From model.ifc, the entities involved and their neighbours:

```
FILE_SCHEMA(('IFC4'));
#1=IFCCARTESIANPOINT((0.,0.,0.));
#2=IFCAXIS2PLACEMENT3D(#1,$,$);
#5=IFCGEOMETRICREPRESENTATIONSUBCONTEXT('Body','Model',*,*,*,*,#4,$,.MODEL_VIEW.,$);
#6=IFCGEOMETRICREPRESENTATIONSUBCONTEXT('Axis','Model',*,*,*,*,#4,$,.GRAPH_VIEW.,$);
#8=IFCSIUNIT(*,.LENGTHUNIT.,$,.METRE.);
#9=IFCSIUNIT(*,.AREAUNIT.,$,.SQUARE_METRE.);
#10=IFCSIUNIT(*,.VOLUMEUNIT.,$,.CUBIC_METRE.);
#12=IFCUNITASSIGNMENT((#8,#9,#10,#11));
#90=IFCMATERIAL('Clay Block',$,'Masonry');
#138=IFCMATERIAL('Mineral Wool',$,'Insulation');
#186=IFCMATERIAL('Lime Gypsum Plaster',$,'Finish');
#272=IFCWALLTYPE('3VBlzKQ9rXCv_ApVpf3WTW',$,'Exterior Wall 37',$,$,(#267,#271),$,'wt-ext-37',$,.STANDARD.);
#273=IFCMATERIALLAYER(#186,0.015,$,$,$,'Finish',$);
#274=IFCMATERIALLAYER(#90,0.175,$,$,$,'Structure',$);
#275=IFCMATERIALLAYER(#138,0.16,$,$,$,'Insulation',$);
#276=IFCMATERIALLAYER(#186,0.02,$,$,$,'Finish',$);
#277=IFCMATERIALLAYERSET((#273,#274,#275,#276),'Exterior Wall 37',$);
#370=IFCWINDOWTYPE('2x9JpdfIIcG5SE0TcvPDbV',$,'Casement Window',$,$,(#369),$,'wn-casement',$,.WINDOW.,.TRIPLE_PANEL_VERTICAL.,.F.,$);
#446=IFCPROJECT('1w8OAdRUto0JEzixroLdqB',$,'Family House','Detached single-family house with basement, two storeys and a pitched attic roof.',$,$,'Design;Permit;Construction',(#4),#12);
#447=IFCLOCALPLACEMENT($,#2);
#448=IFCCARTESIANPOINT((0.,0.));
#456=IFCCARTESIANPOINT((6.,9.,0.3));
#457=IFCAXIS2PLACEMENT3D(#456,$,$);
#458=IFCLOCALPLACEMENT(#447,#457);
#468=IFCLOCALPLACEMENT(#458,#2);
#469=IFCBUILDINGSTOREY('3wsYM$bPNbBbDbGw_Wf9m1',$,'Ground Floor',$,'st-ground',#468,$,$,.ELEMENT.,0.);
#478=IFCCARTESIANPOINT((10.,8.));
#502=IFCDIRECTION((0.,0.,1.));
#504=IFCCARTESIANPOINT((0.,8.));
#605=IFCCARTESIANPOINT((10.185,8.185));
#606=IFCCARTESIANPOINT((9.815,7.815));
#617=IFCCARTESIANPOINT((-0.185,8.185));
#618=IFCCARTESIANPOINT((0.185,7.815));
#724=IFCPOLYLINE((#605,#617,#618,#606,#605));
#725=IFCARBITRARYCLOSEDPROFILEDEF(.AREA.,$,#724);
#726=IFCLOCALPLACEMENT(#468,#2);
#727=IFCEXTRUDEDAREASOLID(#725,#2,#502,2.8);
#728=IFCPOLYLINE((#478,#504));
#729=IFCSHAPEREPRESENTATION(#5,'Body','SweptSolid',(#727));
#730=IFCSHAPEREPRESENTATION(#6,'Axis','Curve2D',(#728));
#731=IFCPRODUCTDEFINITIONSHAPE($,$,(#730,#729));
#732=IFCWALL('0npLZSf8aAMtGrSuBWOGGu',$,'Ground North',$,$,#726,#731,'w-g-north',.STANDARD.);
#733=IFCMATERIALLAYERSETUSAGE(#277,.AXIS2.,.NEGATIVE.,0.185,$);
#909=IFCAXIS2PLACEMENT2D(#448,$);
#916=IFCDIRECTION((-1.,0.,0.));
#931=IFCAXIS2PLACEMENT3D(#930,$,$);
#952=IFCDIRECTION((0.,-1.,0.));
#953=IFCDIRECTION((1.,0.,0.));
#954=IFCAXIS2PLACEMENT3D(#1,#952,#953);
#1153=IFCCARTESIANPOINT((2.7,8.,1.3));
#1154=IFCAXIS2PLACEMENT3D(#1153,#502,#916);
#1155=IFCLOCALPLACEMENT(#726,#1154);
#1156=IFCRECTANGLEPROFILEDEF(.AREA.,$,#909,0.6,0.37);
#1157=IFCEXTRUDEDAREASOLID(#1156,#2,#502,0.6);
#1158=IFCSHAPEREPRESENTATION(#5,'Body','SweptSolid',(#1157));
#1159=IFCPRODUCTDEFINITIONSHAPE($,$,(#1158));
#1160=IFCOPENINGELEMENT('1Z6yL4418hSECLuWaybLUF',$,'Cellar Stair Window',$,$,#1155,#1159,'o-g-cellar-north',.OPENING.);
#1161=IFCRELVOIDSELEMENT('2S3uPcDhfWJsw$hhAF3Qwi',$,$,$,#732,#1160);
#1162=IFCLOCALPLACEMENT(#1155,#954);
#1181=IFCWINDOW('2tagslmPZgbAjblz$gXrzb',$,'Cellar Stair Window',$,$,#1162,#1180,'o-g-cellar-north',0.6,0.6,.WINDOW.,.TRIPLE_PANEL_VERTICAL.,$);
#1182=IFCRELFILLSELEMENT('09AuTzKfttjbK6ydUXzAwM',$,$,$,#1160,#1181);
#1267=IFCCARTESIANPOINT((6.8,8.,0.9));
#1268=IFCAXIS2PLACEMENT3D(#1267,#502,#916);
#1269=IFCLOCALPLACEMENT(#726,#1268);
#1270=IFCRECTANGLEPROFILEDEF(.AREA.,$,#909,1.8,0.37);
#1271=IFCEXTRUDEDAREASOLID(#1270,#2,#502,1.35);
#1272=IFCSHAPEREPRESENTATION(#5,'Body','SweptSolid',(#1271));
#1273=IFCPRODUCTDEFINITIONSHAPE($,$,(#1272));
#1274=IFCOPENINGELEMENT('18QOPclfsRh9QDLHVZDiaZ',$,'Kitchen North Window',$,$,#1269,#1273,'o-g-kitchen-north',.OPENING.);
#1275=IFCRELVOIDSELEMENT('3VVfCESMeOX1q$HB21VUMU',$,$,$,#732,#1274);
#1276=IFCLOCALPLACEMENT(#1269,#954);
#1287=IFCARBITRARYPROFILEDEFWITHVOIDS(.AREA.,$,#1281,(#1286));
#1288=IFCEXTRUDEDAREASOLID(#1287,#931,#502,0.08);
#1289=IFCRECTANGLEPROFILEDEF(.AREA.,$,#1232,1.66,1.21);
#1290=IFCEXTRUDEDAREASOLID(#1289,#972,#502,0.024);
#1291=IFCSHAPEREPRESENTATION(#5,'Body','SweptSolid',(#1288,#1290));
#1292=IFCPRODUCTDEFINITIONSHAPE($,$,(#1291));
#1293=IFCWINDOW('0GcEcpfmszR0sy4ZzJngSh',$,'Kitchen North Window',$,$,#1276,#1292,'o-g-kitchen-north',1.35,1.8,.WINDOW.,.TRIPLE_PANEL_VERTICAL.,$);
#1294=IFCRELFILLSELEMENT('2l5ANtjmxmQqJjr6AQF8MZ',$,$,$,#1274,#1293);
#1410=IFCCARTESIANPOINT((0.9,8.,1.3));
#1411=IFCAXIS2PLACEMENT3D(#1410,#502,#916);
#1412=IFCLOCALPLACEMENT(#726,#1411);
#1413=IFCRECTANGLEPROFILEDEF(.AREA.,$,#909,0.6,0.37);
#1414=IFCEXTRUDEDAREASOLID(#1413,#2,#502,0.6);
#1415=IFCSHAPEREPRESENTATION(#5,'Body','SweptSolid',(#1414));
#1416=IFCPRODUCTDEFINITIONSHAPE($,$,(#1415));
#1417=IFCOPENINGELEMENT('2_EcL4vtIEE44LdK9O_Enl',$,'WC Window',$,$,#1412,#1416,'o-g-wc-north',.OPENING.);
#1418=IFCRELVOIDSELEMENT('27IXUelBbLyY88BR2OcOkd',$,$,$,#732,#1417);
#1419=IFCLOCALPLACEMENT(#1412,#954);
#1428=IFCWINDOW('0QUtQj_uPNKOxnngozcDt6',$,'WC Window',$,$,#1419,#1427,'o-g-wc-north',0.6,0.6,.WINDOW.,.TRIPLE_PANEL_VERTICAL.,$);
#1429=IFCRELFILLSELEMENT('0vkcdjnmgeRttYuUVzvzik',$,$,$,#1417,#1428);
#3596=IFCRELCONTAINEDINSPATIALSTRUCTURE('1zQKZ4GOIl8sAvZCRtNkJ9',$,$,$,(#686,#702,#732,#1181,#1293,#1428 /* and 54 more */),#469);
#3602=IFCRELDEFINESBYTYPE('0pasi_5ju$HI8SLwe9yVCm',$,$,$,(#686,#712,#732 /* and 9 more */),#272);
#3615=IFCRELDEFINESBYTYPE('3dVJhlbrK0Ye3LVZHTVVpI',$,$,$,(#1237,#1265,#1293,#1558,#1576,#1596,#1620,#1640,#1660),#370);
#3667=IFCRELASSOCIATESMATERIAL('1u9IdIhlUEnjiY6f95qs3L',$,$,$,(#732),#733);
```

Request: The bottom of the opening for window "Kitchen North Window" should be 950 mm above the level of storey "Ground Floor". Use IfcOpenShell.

```python
import numpy as np
import ifcopenshell
import ifcopenshell.api.geometry
import ifcopenshell.geom
import ifcopenshell.util.element
import ifcopenshell.util.placement
import ifcopenshell.util.shape
import ifcopenshell.util.unit

model = ifcopenshell.open("model.ifc")
unit_scale = ifcopenshell.util.unit.calculate_unit_scale(model)

window = model.by_id(1293)
opening = window.FillsVoids[0].RelatingOpeningElement
storey = ifcopenshell.util.element.get_container(window, ifc_class="IfcBuildingStorey")
level = ifcopenshell.util.placement.get_local_placement(storey.ObjectPlacement)[2, 3]

# The opening's origin need not be at the sill, so measure its lowest point.
shape = ifcopenshell.geom.create_shape(ifcopenshell.geom.settings(), opening)
bottom = ifcopenshell.util.shape.get_shape_bottom_elevation(shape, shape.geometry) / unit_scale
dz = level + 0.95 / unit_scale - bottom

shift = np.array([0.0, 0.0, dz])
# The window is placed relative to its opening, so it follows when the opening moves.
matrix = ifcopenshell.util.placement.get_local_placement(opening.ObjectPlacement)
matrix[:3, 3] += shift
ifcopenshell.api.geometry.edit_object_placement(
    model, product=opening, matrix=matrix, is_si=False, should_transform_children=True
)

print(f"moved by {dz * unit_scale:+.3f} m")

model.write("model_v2.ifc")
```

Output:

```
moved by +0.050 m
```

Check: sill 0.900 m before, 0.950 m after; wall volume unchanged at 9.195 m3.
